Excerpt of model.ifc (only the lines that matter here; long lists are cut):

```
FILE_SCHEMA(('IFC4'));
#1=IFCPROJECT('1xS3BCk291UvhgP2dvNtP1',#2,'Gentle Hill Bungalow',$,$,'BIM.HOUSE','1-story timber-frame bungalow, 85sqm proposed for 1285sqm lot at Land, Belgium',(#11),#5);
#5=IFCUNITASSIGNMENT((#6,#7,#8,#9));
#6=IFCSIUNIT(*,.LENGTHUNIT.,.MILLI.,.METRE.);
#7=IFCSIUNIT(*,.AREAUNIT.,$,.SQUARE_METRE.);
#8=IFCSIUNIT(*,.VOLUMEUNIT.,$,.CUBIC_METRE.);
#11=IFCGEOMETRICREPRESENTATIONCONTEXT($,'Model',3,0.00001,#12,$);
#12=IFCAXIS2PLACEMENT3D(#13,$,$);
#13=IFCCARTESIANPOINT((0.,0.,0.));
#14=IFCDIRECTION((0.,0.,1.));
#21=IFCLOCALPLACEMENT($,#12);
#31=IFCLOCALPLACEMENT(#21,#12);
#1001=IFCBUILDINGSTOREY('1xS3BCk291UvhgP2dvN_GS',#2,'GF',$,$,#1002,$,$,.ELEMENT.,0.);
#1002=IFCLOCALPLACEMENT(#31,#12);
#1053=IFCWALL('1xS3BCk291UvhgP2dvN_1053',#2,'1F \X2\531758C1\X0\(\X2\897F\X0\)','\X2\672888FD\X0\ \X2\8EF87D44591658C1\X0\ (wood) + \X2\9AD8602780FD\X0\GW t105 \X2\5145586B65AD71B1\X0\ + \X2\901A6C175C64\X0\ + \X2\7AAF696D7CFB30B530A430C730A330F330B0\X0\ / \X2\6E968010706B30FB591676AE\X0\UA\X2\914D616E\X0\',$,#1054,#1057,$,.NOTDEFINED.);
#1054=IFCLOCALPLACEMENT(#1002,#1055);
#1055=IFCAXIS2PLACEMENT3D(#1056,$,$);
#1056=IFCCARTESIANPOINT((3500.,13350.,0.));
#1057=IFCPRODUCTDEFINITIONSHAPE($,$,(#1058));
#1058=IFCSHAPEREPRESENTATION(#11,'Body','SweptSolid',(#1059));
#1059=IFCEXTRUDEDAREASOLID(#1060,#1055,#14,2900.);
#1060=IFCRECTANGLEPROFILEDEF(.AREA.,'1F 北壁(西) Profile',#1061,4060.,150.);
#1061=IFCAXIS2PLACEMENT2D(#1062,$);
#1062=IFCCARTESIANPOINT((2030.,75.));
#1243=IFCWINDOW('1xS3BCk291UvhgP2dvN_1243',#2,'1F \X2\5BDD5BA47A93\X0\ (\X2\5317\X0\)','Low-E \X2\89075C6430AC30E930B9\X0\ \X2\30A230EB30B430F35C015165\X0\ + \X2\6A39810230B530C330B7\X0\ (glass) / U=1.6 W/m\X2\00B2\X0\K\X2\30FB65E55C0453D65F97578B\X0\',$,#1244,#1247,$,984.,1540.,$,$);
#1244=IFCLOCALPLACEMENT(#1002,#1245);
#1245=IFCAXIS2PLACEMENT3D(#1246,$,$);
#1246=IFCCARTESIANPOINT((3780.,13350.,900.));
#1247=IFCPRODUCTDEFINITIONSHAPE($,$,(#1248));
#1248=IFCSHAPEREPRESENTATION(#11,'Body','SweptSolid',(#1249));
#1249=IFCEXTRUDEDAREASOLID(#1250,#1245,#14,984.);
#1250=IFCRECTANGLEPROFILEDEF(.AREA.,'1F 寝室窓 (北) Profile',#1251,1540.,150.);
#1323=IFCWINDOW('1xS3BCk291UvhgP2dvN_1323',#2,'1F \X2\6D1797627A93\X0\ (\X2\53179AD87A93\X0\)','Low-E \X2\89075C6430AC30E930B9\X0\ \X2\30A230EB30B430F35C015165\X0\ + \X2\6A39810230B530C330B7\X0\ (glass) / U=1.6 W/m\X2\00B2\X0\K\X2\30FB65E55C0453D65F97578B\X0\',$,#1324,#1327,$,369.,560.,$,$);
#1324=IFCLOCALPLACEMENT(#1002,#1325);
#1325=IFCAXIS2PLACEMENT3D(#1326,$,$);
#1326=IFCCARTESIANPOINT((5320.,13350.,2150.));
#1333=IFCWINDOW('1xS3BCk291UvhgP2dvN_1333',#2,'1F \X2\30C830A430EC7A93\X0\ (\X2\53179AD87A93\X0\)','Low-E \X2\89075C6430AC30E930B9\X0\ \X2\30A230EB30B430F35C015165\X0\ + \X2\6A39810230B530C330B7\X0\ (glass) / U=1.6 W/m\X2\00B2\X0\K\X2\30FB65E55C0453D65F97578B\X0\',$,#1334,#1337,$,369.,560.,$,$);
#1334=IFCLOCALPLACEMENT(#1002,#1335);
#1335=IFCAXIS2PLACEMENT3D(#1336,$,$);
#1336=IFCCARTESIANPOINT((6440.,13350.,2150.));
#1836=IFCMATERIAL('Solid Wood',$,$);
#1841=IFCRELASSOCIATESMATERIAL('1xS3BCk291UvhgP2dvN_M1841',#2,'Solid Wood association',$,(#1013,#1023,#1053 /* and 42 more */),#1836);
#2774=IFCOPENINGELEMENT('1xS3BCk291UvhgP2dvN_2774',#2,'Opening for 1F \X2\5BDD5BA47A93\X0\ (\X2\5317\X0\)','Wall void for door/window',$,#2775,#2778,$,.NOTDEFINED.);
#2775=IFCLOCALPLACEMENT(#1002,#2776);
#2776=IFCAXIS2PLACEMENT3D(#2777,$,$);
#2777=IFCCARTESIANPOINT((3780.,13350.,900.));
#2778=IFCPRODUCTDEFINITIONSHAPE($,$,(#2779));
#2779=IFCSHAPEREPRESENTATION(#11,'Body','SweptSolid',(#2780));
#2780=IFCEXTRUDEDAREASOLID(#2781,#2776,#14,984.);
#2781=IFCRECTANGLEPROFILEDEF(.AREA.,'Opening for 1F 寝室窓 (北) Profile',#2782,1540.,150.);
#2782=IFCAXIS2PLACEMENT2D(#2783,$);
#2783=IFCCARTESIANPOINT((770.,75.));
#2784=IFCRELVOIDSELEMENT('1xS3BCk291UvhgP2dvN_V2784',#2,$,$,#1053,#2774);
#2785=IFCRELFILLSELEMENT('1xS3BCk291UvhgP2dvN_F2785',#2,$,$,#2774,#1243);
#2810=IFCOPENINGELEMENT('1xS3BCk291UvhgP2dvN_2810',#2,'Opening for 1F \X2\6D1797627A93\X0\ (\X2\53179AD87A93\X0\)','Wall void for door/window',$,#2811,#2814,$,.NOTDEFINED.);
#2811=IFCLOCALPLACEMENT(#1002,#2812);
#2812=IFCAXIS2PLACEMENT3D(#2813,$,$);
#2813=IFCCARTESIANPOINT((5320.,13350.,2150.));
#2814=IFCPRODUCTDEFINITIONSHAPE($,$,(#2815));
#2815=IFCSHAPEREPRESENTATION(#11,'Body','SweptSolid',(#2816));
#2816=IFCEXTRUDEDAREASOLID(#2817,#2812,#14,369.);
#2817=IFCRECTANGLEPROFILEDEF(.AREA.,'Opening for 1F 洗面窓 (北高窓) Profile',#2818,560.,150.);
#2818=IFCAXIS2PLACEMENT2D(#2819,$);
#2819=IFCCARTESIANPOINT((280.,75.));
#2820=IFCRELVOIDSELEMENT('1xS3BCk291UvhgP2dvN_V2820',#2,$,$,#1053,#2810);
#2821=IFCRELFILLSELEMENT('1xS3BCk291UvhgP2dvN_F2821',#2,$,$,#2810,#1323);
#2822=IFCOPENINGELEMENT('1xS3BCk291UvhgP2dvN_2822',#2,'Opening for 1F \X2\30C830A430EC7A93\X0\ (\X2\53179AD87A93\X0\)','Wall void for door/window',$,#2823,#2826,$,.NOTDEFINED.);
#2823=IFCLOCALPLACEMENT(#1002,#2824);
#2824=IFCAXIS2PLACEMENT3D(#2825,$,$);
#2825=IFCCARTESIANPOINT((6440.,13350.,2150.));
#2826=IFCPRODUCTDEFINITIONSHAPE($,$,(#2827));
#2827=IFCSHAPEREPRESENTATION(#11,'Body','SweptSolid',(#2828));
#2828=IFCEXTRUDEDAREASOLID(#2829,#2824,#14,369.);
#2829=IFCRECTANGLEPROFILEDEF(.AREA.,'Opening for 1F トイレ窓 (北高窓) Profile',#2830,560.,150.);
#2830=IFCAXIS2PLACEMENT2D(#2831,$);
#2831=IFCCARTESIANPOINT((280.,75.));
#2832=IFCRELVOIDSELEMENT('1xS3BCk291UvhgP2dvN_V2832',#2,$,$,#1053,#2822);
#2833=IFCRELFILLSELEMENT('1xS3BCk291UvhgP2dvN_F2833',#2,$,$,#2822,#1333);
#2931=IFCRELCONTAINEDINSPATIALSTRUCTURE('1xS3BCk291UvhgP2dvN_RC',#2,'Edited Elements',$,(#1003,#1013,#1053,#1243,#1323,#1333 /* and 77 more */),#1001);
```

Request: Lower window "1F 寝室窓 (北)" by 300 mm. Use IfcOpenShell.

```python
import numpy as np
import ifcopenshell
import ifcopenshell.api.geometry
import ifcopenshell.util.placement
import ifcopenshell.util.unit

model = ifcopenshell.open("model.ifc")
unit_scale = ifcopenshell.util.unit.calculate_unit_scale(model)

window = model.by_guid("1xS3BCk291UvhgP2dvN_1243")
opening = window.FillsVoids[0].RelatingOpeningElement
dz = -0.3 / unit_scale

shift = np.array([0.0, 0.0, dz])
# The window is not placed relative to its opening, so move both.
for product in (opening, window):
    matrix = ifcopenshell.util.placement.get_local_placement(product.ObjectPlacement)
    matrix[:3, 3] += shift
    ifcopenshell.api.geometry.edit_object_placement(model, product=product, matrix=matrix, is_si=False)

print(f"moved by {dz * unit_scale:+.3f} m")

model.write("model_updated.ifc")
```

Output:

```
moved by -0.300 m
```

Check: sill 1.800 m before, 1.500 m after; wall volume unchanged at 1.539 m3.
